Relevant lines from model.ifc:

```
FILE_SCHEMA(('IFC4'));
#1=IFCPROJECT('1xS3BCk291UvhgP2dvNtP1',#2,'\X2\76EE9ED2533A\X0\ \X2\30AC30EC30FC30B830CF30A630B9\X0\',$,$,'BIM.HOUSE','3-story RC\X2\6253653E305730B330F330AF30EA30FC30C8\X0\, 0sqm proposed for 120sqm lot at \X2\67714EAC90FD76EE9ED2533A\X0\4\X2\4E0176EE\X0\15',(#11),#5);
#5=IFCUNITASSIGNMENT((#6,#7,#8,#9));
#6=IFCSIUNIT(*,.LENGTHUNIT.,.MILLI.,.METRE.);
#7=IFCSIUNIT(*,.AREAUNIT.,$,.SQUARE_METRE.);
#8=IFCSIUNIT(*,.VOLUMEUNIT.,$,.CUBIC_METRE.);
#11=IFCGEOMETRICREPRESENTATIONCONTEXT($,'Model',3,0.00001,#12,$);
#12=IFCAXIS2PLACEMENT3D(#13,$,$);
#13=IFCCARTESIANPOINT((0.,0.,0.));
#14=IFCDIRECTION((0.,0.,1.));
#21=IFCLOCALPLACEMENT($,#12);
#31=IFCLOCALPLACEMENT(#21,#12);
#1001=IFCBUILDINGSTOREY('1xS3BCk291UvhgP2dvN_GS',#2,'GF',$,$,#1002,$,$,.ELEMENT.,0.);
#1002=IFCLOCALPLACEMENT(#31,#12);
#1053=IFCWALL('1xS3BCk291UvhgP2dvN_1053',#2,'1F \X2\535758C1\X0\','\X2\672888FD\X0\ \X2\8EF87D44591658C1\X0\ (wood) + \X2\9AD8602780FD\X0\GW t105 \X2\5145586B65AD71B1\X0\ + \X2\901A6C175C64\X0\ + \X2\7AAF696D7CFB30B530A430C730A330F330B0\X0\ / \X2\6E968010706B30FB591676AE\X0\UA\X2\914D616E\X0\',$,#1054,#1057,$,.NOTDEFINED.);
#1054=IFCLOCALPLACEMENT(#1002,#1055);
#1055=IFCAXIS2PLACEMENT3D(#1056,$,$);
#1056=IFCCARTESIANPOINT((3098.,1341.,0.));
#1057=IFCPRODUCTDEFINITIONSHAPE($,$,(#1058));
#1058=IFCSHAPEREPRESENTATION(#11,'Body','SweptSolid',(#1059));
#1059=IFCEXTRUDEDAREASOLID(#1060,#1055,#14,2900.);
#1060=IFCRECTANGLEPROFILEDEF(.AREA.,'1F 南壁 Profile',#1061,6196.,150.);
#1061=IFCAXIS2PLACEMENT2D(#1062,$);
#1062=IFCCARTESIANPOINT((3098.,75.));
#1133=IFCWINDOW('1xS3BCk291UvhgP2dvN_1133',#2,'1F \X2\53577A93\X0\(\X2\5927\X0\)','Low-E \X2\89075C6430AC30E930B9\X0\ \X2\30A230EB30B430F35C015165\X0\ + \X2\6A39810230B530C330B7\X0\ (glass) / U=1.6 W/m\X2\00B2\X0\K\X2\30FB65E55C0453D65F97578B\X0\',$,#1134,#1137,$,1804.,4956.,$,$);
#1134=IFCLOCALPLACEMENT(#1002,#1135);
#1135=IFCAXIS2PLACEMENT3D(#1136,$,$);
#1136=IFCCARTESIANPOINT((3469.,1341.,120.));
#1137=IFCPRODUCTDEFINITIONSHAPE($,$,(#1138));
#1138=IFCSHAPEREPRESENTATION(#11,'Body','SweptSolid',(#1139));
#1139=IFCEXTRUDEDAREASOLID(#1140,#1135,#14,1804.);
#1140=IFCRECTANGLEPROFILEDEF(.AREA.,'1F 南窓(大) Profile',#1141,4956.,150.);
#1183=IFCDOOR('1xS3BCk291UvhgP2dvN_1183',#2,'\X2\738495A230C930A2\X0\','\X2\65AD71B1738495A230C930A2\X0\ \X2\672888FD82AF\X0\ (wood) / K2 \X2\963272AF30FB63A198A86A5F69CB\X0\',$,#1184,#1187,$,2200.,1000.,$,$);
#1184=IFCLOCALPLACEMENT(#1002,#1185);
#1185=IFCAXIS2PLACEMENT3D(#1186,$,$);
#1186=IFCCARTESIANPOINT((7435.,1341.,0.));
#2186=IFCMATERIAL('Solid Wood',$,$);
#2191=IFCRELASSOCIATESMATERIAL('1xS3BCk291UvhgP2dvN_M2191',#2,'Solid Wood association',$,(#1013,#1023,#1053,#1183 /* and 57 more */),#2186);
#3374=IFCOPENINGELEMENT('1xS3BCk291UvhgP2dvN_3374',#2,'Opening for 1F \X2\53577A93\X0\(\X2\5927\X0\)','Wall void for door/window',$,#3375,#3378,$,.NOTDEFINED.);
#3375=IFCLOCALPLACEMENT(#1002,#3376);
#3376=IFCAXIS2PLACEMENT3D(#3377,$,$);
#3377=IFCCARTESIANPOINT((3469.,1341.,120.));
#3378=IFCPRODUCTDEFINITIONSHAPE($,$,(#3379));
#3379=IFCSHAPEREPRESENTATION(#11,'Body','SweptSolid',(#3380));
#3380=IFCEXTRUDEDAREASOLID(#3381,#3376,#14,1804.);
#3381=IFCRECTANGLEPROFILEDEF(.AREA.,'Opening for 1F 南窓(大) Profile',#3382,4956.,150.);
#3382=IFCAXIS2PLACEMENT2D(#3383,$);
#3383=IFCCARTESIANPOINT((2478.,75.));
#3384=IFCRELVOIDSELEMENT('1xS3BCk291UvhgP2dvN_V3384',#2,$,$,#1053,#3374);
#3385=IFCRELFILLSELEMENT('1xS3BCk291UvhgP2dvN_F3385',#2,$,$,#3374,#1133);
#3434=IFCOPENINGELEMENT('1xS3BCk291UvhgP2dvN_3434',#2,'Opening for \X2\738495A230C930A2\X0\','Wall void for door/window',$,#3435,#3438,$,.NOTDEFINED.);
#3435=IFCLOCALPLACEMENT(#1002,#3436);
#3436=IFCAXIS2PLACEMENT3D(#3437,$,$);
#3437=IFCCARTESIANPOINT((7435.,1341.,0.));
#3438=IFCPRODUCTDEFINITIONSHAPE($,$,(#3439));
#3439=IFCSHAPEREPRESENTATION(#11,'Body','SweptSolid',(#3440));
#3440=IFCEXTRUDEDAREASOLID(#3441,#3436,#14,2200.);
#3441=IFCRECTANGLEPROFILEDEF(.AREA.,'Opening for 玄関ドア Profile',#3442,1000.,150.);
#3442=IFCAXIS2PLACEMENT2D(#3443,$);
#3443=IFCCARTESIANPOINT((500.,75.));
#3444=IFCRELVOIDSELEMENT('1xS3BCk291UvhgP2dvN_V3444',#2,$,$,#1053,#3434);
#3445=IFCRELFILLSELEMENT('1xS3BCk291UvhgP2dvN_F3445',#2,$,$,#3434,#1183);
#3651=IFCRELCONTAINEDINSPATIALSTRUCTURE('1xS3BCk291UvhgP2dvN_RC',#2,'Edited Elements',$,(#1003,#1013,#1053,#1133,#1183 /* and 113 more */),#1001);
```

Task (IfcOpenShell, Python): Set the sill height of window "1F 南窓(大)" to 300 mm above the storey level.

```python
import numpy as np
import ifcopenshell
import ifcopenshell.api.geometry
import ifcopenshell.geom
import ifcopenshell.util.element
import ifcopenshell.util.placement
import ifcopenshell.util.shape
import ifcopenshell.util.unit

model = ifcopenshell.open("model.ifc")
unit_scale = ifcopenshell.util.unit.calculate_unit_scale(model)

window = model.by_guid("1xS3BCk291UvhgP2dvN_1133")
opening = window.FillsVoids[0].RelatingOpeningElement
storey = ifcopenshell.util.element.get_container(window, ifc_class="IfcBuildingStorey")
level = ifcopenshell.util.placement.get_local_placement(storey.ObjectPlacement)[2, 3]

# The opening's origin need not be at the sill, so measure its lowest point.
shape = ifcopenshell.geom.create_shape(ifcopenshell.geom.settings(), opening)
bottom = ifcopenshell.util.shape.get_shape_bottom_elevation(shape, shape.geometry) / unit_scale
dz = level + 0.3 / unit_scale - bottom

shift = np.array([0.0, 0.0, dz])
# The window is not placed relative to its opening, so move both.
for product in (opening, window):
    matrix = ifcopenshell.util.placement.get_local_placement(product.ObjectPlacement)
    matrix[:3, 3] += shift
    ifcopenshell.api.geometry.edit_object_placement(model, product=product, matrix=matrix, is_si=False)

print(f"moved by {dz * unit_scale:+.3f} m")

model.write("model_rev.ifc")
```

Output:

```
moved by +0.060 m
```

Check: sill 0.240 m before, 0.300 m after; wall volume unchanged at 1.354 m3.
